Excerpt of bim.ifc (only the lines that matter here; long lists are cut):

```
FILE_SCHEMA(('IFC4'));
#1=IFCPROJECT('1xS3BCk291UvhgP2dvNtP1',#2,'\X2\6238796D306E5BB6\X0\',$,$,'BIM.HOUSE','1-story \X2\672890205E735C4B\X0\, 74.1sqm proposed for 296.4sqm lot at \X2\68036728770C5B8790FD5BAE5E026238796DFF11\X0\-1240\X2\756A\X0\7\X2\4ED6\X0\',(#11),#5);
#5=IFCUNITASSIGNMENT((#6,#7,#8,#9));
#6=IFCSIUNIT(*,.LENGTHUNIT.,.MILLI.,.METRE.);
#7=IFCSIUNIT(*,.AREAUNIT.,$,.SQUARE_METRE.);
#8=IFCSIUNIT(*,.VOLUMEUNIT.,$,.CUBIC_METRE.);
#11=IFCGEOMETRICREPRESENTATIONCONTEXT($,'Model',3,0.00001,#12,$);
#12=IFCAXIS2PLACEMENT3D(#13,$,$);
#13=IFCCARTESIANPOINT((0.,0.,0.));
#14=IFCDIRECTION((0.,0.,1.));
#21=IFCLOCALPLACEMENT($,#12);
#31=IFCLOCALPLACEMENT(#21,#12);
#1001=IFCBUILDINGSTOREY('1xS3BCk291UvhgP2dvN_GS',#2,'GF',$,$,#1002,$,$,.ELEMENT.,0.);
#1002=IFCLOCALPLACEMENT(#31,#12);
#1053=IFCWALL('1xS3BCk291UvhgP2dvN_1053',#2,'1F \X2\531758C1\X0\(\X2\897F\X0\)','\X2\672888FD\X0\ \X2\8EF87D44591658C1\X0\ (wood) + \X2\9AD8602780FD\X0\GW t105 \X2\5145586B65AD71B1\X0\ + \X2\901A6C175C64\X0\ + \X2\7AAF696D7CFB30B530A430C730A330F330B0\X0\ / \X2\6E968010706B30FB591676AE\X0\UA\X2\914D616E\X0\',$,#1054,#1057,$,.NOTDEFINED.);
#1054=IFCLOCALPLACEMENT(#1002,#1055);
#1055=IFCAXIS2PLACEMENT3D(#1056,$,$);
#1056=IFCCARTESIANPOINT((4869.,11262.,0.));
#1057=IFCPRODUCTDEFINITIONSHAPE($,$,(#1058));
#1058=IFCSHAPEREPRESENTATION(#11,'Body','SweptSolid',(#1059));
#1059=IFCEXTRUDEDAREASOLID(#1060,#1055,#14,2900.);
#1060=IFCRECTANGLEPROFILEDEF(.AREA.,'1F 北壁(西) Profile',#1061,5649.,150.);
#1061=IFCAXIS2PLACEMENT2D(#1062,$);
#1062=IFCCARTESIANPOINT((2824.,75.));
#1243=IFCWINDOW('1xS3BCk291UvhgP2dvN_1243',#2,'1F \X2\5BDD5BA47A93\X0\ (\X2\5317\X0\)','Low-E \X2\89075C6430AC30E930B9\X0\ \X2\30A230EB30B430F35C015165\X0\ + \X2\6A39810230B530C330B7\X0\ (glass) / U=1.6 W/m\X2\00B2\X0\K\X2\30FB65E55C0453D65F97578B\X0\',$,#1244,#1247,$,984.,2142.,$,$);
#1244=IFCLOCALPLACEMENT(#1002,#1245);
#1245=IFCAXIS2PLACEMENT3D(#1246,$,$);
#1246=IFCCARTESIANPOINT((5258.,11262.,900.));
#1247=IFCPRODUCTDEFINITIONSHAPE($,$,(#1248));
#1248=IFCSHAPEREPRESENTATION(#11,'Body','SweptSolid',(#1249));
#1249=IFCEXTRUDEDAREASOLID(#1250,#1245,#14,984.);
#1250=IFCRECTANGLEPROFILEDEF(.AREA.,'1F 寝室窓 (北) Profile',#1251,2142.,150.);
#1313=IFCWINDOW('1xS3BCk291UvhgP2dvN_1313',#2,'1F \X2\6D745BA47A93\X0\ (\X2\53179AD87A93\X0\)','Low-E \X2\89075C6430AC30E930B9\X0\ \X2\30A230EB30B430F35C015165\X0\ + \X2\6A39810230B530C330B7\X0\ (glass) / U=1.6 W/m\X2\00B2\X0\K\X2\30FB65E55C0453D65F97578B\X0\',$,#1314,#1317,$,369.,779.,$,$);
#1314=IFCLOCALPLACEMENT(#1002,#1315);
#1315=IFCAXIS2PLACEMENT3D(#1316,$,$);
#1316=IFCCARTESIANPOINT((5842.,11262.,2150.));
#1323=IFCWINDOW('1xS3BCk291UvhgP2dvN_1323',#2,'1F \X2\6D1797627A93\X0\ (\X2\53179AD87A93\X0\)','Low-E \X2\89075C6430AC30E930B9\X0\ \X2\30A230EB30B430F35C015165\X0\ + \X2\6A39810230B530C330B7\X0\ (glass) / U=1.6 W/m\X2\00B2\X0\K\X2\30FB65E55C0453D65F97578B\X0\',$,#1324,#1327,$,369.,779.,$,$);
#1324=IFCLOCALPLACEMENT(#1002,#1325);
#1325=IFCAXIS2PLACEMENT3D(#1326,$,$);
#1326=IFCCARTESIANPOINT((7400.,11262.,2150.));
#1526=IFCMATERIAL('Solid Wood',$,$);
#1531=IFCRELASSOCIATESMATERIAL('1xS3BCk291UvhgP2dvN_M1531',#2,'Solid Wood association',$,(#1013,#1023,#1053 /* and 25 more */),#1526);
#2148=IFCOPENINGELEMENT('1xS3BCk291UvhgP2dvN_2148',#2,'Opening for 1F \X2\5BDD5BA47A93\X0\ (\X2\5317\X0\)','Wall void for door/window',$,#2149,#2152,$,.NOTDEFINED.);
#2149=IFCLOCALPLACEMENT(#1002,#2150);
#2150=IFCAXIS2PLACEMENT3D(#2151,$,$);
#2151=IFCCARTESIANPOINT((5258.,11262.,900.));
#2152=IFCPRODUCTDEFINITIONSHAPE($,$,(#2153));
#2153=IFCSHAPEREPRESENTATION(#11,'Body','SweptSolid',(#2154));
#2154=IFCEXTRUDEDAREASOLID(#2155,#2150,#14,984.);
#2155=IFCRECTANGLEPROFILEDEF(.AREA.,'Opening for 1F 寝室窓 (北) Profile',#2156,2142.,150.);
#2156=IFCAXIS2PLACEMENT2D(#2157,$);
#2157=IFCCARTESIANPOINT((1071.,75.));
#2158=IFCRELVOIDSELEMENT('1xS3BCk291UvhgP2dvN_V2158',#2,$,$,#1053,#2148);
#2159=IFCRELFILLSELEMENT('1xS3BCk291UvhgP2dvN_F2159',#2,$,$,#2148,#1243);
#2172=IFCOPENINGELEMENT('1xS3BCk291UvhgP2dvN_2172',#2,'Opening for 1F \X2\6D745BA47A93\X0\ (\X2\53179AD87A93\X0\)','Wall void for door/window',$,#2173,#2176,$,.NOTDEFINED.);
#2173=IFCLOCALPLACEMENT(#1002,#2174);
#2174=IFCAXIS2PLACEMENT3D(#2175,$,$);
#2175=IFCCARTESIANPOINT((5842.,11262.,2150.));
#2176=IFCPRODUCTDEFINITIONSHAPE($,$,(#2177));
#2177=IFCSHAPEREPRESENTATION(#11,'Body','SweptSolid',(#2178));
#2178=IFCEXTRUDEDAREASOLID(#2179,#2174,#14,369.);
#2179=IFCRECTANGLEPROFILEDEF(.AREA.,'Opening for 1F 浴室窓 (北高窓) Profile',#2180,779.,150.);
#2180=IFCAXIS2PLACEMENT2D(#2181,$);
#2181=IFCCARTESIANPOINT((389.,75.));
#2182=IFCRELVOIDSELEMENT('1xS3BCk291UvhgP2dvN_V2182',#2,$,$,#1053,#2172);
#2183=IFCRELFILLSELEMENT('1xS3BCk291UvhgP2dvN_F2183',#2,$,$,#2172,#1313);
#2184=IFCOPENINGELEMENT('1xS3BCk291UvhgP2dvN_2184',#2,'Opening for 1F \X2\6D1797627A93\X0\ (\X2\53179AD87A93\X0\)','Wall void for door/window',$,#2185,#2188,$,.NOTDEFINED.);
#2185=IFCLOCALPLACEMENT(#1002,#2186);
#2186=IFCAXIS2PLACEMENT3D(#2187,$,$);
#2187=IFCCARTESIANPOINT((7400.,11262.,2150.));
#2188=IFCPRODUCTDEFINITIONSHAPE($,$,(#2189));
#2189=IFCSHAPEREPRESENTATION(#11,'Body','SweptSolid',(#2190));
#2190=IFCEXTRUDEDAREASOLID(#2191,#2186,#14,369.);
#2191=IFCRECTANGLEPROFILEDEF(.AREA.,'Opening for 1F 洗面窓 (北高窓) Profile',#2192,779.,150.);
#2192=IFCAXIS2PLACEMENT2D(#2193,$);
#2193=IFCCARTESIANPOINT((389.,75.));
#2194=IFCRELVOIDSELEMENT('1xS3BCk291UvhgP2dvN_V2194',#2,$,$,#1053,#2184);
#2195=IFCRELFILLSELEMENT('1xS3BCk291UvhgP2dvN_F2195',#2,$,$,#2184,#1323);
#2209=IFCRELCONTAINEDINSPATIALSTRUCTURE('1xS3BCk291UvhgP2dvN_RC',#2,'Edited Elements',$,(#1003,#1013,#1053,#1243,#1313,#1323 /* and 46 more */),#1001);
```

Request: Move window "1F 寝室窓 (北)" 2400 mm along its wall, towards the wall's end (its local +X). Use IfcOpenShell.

```python
import ifcopenshell
import ifcopenshell.api.geometry
import ifcopenshell.util.placement

model = ifcopenshell.open("bim.ifc")

window = model.by_guid("1xS3BCk291UvhgP2dvN_1243")
opening = window.FillsVoids[0].RelatingOpeningElement
wall = opening.VoidsElements[0].RelatingBuildingElement

wall_matrix = ifcopenshell.util.placement.get_local_placement(wall.ObjectPlacement)
shift = wall_matrix[:3, 0] * 2400.0
before = ifcopenshell.util.placement.get_local_placement(window.ObjectPlacement)[:3, 3].copy()

# The window is not placed relative to its opening, so move both.
for product in (opening, window):
    matrix = ifcopenshell.util.placement.get_local_placement(product.ObjectPlacement)
    matrix[:3, 3] += shift
    ifcopenshell.api.geometry.edit_object_placement(model, product=product, matrix=matrix, is_si=False)

after = ifcopenshell.util.placement.get_local_placement(window.ObjectPlacement)[:3, 3]
print("window moved by", (after - before).round(3) + 0.0)

model.write("bim-out.ifc")
```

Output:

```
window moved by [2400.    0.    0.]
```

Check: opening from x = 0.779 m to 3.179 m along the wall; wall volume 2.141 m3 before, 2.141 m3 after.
